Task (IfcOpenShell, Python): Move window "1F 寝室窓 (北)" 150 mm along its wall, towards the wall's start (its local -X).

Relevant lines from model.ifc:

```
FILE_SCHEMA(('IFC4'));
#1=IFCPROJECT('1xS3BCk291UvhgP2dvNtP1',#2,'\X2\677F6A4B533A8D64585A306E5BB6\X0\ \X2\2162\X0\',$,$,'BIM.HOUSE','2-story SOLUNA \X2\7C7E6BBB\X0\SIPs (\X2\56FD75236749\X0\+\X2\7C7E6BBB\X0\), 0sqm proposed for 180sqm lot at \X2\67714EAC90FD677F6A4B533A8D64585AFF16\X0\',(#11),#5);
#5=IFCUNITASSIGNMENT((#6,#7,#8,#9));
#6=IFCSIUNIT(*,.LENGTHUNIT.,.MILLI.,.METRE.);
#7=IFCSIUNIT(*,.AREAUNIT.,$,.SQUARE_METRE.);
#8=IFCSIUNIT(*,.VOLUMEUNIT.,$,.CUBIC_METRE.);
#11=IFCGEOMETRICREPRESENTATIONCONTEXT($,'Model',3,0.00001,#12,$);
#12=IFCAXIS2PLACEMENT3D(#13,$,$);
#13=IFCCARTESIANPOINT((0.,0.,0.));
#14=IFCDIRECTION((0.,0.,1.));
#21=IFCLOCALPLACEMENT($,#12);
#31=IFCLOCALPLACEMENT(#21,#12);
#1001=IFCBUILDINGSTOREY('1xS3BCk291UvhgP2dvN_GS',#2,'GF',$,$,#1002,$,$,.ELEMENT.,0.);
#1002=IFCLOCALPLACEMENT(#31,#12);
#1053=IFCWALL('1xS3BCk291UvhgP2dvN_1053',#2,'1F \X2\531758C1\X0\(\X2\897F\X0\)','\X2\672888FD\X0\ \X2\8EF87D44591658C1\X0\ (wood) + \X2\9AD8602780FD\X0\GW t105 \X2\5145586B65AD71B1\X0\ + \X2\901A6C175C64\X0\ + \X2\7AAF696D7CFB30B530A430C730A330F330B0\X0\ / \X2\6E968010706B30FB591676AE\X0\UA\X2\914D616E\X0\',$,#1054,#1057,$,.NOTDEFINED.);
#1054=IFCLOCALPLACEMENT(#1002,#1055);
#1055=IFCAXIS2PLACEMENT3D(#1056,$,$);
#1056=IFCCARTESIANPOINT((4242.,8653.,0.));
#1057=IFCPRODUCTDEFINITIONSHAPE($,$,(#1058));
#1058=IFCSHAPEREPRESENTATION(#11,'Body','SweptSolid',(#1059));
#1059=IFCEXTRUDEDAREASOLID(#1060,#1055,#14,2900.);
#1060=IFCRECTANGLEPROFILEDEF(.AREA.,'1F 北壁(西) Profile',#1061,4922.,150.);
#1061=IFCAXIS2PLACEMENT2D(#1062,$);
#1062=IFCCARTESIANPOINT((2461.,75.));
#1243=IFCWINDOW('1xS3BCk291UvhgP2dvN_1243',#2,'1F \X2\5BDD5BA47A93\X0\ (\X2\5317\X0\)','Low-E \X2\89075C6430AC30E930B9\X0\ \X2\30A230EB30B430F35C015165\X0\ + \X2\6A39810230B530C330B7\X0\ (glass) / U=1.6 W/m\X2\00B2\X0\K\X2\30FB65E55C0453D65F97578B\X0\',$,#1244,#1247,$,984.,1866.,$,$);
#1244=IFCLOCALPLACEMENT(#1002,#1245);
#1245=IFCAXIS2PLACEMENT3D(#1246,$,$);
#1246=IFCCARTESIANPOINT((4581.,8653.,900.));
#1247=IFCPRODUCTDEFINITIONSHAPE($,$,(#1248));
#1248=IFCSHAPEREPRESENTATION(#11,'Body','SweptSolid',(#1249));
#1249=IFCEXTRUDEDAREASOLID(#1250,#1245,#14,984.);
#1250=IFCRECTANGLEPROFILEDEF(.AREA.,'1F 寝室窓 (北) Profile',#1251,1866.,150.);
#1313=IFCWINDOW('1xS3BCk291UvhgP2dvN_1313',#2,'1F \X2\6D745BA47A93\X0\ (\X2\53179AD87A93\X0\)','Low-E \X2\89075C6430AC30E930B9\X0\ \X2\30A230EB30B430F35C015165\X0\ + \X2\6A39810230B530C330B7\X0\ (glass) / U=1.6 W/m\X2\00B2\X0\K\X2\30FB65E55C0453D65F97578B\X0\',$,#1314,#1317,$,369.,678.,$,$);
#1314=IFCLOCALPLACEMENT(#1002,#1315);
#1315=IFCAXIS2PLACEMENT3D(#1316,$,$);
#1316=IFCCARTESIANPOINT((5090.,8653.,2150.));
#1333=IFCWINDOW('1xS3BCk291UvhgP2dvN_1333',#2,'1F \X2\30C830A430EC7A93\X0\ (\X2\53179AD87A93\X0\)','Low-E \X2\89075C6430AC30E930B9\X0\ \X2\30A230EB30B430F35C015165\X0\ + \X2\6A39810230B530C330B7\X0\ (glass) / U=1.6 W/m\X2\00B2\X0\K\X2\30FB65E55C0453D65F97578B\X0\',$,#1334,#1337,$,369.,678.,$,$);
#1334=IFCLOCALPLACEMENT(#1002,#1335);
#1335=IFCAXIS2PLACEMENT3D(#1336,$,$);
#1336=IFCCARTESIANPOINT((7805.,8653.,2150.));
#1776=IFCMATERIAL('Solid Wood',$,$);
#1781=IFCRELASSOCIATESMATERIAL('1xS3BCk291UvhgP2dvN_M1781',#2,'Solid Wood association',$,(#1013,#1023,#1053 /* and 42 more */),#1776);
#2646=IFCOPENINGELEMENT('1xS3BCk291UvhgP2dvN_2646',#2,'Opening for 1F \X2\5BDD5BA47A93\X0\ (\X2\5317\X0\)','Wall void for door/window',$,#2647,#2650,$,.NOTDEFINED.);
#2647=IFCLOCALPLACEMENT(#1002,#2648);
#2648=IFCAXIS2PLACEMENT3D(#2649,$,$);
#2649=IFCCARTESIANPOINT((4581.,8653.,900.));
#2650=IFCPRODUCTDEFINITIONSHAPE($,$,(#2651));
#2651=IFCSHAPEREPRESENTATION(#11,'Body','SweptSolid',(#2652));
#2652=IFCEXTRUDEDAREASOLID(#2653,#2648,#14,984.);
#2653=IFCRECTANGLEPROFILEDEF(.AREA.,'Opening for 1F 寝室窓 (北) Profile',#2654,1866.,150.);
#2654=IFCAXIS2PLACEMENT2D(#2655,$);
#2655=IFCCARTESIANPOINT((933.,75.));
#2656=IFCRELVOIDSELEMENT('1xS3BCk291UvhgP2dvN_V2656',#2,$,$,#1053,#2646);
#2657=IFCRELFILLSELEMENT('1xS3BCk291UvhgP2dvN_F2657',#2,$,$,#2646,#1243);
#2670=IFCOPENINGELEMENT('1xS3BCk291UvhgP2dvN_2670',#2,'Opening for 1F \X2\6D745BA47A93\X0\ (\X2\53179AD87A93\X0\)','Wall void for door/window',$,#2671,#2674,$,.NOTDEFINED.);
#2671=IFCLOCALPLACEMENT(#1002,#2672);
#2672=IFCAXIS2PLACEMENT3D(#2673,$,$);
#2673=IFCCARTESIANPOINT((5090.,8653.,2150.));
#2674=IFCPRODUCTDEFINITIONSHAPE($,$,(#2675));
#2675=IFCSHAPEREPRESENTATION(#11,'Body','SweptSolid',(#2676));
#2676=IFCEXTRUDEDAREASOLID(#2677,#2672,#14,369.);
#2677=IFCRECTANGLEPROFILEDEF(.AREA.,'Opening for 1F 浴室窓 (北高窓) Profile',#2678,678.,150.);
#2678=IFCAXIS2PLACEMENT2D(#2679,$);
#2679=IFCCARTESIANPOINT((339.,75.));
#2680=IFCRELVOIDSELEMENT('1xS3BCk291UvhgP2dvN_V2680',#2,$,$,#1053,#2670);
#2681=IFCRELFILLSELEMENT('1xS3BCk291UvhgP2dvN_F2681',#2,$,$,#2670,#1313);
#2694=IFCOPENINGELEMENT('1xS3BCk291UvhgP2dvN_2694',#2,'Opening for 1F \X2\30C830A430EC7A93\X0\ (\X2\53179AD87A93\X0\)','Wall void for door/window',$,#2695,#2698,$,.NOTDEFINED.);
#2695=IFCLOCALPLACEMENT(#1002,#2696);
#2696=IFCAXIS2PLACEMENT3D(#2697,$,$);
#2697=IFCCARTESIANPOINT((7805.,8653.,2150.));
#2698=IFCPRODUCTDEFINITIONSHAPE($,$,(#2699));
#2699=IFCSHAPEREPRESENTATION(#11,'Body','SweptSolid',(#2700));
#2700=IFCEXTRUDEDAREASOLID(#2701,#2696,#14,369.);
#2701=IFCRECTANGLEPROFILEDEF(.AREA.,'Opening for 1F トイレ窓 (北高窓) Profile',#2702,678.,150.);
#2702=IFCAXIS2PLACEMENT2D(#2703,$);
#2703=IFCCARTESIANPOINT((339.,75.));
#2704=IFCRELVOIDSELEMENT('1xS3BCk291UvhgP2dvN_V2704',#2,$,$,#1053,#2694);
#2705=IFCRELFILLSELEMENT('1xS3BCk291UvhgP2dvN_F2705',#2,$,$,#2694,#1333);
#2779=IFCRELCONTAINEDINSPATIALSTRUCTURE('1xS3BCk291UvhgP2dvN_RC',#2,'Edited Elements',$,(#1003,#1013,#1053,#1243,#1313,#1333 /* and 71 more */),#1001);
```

```python
import ifcopenshell
import ifcopenshell.api.geometry
import ifcopenshell.util.placement
import ifcopenshell.util.unit

model = ifcopenshell.open("model.ifc")
unit_scale = ifcopenshell.util.unit.calculate_unit_scale(model)

window = model.by_guid("1xS3BCk291UvhgP2dvN_1243")
opening = window.FillsVoids[0].RelatingOpeningElement
wall = opening.VoidsElements[0].RelatingBuildingElement

wall_matrix = ifcopenshell.util.placement.get_local_placement(wall.ObjectPlacement)
shift = wall_matrix[:3, 0] * -0.15 / unit_scale
before = ifcopenshell.util.placement.get_local_placement(window.ObjectPlacement)[:3, 3].copy()

# The window is not placed relative to its opening, so move both.
for product in (opening, window):
    matrix = ifcopenshell.util.placement.get_local_placement(product.ObjectPlacement)
    matrix[:3, 3] += shift
    ifcopenshell.api.geometry.edit_object_placement(model, product=product, matrix=matrix, is_si=False)

after = ifcopenshell.util.placement.get_local_placement(window.ObjectPlacement)[:3, 3]
print("window moved by", (after - before).round(3) + 0.0)

model.write("model_edited.ifc")
```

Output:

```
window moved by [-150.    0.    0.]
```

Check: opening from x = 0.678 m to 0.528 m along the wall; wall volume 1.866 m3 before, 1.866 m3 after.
